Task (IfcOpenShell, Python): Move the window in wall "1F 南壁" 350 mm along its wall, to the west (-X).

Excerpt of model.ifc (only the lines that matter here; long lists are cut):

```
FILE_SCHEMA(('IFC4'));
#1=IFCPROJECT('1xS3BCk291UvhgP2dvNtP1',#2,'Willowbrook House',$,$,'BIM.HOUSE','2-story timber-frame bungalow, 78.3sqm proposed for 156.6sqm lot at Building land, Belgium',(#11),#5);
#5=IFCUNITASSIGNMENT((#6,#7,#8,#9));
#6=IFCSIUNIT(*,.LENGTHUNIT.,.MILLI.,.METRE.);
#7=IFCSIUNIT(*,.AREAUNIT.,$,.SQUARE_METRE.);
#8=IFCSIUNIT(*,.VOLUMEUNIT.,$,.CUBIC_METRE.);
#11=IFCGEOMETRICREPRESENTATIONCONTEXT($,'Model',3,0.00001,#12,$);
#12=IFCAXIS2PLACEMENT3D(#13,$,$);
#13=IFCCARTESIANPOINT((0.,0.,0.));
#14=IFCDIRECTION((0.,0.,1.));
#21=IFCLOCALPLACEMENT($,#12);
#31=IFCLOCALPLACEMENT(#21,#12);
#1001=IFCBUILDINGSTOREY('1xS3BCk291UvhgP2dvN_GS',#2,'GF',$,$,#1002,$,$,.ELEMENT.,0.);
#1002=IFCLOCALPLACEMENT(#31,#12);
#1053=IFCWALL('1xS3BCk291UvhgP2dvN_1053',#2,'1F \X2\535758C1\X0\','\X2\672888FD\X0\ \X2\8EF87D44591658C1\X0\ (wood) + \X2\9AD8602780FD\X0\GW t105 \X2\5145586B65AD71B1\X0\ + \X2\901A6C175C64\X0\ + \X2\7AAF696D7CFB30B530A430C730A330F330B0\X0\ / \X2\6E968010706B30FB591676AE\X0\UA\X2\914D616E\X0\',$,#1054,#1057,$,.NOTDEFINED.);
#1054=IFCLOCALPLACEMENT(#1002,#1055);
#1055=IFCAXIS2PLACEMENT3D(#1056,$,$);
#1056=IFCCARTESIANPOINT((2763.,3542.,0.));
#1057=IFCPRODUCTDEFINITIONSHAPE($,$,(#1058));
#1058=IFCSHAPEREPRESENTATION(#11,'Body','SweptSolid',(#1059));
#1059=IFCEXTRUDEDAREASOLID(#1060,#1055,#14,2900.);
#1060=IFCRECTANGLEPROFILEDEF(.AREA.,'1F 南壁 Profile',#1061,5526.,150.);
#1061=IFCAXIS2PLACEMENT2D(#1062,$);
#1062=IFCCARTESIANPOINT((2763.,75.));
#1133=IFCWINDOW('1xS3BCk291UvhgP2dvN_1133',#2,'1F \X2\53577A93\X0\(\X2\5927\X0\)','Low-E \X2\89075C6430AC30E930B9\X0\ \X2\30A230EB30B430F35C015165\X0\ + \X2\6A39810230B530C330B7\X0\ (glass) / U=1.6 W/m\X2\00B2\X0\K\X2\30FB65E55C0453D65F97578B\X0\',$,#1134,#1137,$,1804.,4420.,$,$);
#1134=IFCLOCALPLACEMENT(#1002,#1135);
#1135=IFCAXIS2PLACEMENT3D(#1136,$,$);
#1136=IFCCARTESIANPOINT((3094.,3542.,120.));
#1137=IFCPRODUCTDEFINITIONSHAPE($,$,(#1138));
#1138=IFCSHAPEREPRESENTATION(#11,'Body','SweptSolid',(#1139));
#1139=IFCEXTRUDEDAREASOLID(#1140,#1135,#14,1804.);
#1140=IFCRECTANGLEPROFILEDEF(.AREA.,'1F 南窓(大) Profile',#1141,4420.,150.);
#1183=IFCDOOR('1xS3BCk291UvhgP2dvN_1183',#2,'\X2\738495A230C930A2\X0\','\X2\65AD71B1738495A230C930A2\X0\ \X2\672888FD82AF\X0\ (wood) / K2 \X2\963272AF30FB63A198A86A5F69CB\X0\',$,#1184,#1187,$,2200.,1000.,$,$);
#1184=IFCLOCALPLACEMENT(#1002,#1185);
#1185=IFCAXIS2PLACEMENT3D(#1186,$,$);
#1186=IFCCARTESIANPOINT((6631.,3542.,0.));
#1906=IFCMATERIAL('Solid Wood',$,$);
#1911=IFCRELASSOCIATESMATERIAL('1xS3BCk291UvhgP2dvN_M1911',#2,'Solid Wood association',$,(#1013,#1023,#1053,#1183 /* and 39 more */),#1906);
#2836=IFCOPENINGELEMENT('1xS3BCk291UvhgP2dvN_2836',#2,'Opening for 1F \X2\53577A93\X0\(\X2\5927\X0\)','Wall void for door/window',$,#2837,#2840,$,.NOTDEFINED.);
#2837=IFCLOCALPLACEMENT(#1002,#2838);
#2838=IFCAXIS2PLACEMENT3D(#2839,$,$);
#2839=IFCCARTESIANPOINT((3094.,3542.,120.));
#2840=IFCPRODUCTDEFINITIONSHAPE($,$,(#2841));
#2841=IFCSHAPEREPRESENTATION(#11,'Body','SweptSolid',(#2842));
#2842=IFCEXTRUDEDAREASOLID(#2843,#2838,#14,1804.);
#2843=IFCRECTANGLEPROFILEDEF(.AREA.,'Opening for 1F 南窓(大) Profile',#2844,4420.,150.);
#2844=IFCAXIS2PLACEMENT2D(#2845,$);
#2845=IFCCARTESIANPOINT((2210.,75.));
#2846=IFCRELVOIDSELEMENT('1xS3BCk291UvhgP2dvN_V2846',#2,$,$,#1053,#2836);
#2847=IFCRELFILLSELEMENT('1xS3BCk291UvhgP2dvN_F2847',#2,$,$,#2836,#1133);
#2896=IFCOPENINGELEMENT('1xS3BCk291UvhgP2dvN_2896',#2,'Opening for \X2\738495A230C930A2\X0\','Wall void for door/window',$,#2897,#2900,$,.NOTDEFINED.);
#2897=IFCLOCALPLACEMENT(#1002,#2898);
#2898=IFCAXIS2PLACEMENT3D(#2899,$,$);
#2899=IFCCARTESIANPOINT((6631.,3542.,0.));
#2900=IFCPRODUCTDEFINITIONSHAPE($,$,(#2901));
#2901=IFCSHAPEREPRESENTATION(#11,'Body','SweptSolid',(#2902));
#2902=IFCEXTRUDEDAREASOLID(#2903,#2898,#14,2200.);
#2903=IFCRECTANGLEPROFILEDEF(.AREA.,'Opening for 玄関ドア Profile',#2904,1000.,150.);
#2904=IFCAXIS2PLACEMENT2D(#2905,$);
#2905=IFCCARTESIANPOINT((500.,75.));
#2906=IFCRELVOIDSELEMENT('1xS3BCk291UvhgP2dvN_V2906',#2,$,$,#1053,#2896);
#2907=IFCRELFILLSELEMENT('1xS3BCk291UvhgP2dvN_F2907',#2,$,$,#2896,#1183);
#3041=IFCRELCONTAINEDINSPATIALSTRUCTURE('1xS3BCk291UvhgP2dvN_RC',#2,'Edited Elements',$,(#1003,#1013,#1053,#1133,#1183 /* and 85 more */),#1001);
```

```python
import ifcopenshell
import ifcopenshell.api.geometry
import ifcopenshell.util.placement

model = ifcopenshell.open("model.ifc")

window = model.by_guid("1xS3BCk291UvhgP2dvN_1133")
opening = window.FillsVoids[0].RelatingOpeningElement
wall = opening.VoidsElements[0].RelatingBuildingElement

wall_matrix = ifcopenshell.util.placement.get_local_placement(wall.ObjectPlacement)
shift = wall_matrix[:3, 0] * -350.0
before = ifcopenshell.util.placement.get_local_placement(window.ObjectPlacement)[:3, 3].copy()

# The window is not placed relative to its opening, so move both.
for product in (opening, window):
    matrix = ifcopenshell.util.placement.get_local_placement(product.ObjectPlacement)
    matrix[:3, 3] += shift
    ifcopenshell.api.geometry.edit_object_placement(model, product=product, matrix=matrix, is_si=False)

after = ifcopenshell.util.placement.get_local_placement(window.ObjectPlacement)[:3, 3]
print("window moved by", (after - before).round(3) + 0.0)

model.write("model_rev.ifc")
```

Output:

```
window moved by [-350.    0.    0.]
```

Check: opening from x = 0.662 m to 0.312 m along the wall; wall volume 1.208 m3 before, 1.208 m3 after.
